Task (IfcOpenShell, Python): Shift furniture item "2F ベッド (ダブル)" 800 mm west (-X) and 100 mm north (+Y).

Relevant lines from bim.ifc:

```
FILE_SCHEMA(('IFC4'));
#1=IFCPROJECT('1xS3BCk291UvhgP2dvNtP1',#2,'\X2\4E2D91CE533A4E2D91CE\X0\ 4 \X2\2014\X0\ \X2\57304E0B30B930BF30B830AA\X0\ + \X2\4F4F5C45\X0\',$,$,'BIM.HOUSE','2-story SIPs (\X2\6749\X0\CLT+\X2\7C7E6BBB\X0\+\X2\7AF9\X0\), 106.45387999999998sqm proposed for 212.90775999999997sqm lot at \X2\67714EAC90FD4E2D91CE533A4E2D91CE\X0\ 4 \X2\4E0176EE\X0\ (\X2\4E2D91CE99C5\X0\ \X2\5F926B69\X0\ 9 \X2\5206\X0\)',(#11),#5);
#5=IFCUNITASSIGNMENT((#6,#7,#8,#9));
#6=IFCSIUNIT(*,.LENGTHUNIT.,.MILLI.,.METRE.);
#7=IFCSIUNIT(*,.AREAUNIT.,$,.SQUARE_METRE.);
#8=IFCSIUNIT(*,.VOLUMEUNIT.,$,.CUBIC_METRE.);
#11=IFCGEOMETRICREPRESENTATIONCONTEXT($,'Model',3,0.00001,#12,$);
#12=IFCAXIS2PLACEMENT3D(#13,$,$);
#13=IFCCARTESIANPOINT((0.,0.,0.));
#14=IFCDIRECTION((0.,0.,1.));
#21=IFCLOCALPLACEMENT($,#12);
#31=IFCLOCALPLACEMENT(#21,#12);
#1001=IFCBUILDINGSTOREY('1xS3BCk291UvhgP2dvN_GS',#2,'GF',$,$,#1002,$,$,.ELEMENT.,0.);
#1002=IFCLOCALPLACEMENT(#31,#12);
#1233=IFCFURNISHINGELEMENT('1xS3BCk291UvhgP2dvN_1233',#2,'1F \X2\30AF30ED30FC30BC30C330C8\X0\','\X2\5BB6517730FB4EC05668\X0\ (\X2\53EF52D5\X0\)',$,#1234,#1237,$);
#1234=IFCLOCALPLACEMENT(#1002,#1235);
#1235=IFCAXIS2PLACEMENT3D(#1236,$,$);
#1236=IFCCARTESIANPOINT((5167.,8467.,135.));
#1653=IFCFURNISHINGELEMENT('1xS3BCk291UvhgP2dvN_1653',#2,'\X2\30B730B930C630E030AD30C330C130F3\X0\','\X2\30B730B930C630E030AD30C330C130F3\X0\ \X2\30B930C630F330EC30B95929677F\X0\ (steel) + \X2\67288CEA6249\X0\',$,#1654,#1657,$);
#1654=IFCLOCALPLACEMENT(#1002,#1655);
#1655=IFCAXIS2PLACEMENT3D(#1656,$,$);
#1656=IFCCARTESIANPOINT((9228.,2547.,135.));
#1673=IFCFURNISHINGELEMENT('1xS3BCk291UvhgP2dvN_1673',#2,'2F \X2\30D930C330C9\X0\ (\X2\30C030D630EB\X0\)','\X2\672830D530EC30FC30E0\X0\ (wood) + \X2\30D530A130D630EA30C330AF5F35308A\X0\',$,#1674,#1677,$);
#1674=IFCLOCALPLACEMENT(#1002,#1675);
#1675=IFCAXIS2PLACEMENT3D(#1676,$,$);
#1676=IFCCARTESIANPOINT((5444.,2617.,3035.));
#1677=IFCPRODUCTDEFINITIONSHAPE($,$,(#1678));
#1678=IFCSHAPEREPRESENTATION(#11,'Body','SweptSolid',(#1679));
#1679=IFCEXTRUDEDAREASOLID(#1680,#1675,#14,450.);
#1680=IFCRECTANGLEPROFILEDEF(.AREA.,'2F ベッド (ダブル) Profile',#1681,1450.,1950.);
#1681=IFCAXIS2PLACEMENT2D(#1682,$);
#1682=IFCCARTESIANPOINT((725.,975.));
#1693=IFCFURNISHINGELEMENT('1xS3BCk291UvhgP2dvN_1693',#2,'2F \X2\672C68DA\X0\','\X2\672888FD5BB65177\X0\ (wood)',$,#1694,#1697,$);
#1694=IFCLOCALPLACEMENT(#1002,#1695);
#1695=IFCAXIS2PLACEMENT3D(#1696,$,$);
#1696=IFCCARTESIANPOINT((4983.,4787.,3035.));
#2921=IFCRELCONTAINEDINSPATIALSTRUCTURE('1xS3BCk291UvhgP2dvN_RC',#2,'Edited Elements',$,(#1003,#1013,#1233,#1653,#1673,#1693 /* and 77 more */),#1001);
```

```python
import ifcopenshell
import ifcopenshell.api.geometry
import ifcopenshell.util.placement

model = ifcopenshell.open("bim.ifc")

item = model.by_guid("1xS3BCk291UvhgP2dvN_1673")
matrix = ifcopenshell.util.placement.get_local_placement(item.ObjectPlacement)
matrix[0, 3] -= 800.0
matrix[1, 3] += 100.0
ifcopenshell.api.geometry.edit_object_placement(model, product=item, matrix=matrix, is_si=False)

print(ifcopenshell.util.placement.get_local_placement(item.ObjectPlacement).round(3) + 0.0)

model.write("bim_rev.ifc")
```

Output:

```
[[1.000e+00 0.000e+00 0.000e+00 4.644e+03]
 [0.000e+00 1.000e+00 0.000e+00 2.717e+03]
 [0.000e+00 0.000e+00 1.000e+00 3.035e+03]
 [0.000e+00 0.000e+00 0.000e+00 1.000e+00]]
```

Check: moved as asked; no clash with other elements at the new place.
